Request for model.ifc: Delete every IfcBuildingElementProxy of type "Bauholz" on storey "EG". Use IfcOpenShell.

First a look at what the model holds.

```python
import ifcopenshell
import ifcopenshell.util.element

model = ifcopenshell.open("model.ifc")
print(model.schema)
storey = next(s for s in model.by_type("IfcBuildingStorey") if s.Name == "EG")
proxies = [e for e in ifcopenshell.util.element.get_decomposition(storey) if e.is_a("IfcBuildingElementProxy")]
seen = {}
for e in proxies:
    element_type = ifcopenshell.util.element.get_type(e)
    name = element_type.Name if element_type not in (None, e) else None
    seen[name] = seen.get(name, 0) + 1
for name, count in sorted(seen.items(), key=str):
    print(count, "x", name)
```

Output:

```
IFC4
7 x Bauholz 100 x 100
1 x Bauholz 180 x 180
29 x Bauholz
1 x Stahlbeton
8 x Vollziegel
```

```python
import ifcopenshell
import ifcopenshell.api.root
import ifcopenshell.util.element

model = ifcopenshell.open("model.ifc")

storey = next(s for s in model.by_type("IfcBuildingStorey") if s.Name == "EG")
proxies = [e for e in ifcopenshell.util.element.get_decomposition(storey) if e.is_a("IfcBuildingElementProxy")]
targets = [e for e in proxies if (t := ifcopenshell.util.element.get_type(e)) not in (None, e) and t.Name == "Bauholz"]

for e in targets:
    ifcopenshell.api.root.remove_product(model, product=e)
print(len(targets), "removed")

model.write("model_rev.ifc")
```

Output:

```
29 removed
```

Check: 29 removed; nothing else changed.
